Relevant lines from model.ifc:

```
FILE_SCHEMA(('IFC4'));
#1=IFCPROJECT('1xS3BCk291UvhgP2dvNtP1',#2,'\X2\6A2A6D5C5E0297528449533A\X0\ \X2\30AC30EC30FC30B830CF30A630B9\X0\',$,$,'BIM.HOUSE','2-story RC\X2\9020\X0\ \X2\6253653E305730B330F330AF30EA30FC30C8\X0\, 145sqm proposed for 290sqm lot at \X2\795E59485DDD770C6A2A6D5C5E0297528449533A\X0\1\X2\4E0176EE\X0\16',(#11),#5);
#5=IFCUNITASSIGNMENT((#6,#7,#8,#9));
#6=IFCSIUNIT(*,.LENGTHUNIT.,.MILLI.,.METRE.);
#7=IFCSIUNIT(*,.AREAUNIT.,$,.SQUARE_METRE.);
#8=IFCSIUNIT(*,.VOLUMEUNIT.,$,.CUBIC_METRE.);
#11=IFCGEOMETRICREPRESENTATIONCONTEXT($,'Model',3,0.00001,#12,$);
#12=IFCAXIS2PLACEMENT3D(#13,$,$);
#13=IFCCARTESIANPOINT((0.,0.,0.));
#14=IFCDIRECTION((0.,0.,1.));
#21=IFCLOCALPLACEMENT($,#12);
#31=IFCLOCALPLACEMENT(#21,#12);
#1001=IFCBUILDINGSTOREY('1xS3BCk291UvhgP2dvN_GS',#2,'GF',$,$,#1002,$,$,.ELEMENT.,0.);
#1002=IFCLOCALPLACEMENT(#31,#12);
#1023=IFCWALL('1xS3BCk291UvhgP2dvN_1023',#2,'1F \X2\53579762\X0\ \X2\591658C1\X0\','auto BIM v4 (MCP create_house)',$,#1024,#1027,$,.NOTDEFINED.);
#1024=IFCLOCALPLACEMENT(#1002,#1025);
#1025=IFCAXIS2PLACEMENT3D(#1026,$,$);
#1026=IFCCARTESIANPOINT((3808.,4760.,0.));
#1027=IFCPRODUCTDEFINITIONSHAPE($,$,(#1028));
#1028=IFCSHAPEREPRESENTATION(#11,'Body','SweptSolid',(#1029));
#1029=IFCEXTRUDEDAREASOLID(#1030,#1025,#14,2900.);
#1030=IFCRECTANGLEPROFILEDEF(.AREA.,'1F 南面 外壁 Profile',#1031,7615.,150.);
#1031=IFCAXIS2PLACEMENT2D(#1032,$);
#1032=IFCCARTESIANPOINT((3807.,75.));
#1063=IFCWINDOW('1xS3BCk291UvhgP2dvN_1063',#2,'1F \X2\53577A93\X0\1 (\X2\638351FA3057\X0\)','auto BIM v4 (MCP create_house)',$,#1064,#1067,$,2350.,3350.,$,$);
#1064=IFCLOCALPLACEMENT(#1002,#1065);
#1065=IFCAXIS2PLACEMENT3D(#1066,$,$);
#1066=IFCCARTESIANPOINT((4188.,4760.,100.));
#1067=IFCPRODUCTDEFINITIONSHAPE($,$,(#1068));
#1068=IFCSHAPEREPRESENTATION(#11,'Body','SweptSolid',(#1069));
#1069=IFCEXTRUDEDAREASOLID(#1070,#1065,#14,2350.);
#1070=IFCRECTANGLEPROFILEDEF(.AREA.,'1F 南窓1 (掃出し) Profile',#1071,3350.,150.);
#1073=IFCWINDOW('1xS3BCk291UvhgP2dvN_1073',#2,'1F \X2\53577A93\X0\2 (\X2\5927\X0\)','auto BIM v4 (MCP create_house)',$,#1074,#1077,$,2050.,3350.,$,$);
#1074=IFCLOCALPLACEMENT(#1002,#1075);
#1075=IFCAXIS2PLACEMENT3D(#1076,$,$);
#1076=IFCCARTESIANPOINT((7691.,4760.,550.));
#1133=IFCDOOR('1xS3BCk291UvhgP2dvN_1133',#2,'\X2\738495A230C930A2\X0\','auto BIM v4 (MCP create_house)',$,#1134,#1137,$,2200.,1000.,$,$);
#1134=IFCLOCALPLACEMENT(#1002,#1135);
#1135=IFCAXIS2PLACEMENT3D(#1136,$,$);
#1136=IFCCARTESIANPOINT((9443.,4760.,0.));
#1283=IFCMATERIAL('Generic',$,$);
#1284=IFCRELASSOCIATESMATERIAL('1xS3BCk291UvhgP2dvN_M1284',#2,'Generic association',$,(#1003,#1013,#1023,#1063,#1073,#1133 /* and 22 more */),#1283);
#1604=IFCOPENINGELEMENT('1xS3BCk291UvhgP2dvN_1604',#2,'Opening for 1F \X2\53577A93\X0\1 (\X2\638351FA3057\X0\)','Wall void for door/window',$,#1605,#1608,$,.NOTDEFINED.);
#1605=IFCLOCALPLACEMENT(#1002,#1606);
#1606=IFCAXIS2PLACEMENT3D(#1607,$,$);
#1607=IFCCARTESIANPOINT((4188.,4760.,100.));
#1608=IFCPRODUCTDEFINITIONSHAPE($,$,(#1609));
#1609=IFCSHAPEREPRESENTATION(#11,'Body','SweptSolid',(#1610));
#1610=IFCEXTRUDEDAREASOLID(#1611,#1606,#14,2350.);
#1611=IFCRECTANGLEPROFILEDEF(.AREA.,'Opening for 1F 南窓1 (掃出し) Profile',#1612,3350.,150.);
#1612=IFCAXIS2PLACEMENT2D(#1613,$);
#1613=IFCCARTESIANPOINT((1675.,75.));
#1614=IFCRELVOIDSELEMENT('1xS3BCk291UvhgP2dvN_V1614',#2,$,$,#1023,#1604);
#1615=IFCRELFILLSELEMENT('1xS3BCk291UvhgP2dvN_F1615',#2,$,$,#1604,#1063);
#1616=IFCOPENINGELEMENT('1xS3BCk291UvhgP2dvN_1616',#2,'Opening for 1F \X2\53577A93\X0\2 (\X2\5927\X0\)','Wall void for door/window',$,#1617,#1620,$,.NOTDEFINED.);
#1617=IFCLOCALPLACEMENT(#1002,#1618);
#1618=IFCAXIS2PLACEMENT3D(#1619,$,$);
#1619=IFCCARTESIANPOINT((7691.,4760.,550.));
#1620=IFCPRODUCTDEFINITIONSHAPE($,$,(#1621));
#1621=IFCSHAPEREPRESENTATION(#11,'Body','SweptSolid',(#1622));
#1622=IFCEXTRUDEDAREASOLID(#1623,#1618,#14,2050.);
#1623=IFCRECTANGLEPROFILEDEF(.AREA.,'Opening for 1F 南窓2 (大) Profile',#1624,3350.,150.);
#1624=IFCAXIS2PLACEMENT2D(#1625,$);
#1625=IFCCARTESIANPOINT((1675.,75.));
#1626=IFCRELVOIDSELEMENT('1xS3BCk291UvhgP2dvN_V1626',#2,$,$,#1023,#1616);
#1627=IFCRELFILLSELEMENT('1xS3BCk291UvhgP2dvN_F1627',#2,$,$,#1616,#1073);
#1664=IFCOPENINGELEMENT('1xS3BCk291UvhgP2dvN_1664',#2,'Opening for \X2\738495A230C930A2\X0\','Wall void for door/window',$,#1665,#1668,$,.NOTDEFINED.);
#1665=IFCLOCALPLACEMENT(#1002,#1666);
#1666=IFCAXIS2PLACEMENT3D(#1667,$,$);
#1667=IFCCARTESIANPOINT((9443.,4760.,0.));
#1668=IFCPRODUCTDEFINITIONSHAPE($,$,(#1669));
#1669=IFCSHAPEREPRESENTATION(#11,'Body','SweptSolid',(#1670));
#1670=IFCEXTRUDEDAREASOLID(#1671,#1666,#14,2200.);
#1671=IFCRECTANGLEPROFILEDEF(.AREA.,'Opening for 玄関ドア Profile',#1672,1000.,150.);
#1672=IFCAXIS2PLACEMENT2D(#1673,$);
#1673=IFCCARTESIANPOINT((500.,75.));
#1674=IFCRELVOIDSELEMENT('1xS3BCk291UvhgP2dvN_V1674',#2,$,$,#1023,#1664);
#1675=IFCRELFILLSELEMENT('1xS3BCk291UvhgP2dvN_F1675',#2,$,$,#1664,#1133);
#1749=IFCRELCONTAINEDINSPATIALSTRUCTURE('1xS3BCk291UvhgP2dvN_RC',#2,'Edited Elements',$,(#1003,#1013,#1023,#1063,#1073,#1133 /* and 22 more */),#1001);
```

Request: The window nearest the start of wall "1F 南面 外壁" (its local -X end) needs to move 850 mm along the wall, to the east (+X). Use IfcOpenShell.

```python
import ifcopenshell
import ifcopenshell.api.geometry
import ifcopenshell.util.placement
import ifcopenshell.util.unit

model = ifcopenshell.open("model.ifc")
unit_scale = ifcopenshell.util.unit.calculate_unit_scale(model)

window = model.by_guid("1xS3BCk291UvhgP2dvN_1063")
opening = window.FillsVoids[0].RelatingOpeningElement
wall = opening.VoidsElements[0].RelatingBuildingElement

wall_matrix = ifcopenshell.util.placement.get_local_placement(wall.ObjectPlacement)
shift = wall_matrix[:3, 0] * 0.85 / unit_scale
before = ifcopenshell.util.placement.get_local_placement(window.ObjectPlacement)[:3, 3].copy()

# The window is not placed relative to its opening, so move both.
for product in (opening, window):
    matrix = ifcopenshell.util.placement.get_local_placement(product.ObjectPlacement)
    matrix[:3, 3] += shift
    ifcopenshell.api.geometry.edit_object_placement(model, product=product, matrix=matrix, is_si=False)

after = ifcopenshell.util.placement.get_local_placement(window.ObjectPlacement)[:3, 3]
print("window moved by", (after - before).round(3) + 0.0)

model.write("model-out.ifc")
```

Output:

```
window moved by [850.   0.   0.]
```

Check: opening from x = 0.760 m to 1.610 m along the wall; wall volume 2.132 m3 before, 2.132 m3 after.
